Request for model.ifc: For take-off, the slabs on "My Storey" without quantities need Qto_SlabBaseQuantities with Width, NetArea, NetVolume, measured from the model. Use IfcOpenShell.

First a look at what the model holds.

```python
import ifcopenshell
import ifcopenshell.util.element
import ifcopenshell.util.unit

model = ifcopenshell.open("model.ifc")
print(model.schema)
for unit_type in ("LENGTHUNIT", "AREAUNIT", "VOLUMEUNIT"):
    print(unit_type, ifcopenshell.util.unit.calculate_unit_scale(model, unit_type))
storey = next(s for s in model.by_type("IfcBuildingStorey") if s.Name == "My Storey")
slabs = [e for e in ifcopenshell.util.element.get_decomposition(storey) if e.is_a("IfcSlab")]
for e in sorted(slabs, key=lambda e: e.id()):
    print(e.id(), e.is_a(), e.Name, list(ifcopenshell.util.element.get_psets(e, qtos_only=True)), sep=" | ")
```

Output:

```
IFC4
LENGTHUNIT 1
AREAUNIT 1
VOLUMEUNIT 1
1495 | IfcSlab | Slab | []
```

```python
import ifcopenshell
import ifcopenshell.api.pset
import ifcopenshell.geom
import ifcopenshell.util.element
import ifcopenshell.util.shape
import ifcopenshell.util.unit

model = ifcopenshell.open("model.ifc")
unit_scale = ifcopenshell.util.unit.calculate_unit_scale(model)
area_scale = ifcopenshell.util.unit.calculate_unit_scale(model, "AREAUNIT")
volume_scale = ifcopenshell.util.unit.calculate_unit_scale(model, "VOLUMEUNIT")
settings = ifcopenshell.geom.settings()

storey = next(s for s in model.by_type("IfcBuildingStorey") if s.Name == "My Storey")
slabs = [e for e in ifcopenshell.util.element.get_decomposition(storey) if e.is_a("IfcSlab")]

for e in sorted(slabs, key=lambda e: e.id()):
    if ifcopenshell.util.element.get_psets(e, qtos_only=True, should_inherit=False):
        continue
    # Geometry comes back in metres, in the element's own axes.
    shape = ifcopenshell.geom.create_shape(settings, e)
    values = {
        "Width": ifcopenshell.util.shape.get_z(shape.geometry) / unit_scale,
        "NetArea": ifcopenshell.util.shape.get_footprint_area(shape.geometry) / area_scale,
        "NetVolume": ifcopenshell.util.shape.get_volume(shape.geometry) / volume_scale,
    }
    qto = ifcopenshell.api.pset.add_qto(model, product=e, name="Qto_SlabBaseQuantities")
    ifcopenshell.api.pset.edit_qto(model, qto=qto, properties=values)
    print(e.id(), {k: round(v, 3) for k, v in values.items()})

model.write("model_v2.ifc")
```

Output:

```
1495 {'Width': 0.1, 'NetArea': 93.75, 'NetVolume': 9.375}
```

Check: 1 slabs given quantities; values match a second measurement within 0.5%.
